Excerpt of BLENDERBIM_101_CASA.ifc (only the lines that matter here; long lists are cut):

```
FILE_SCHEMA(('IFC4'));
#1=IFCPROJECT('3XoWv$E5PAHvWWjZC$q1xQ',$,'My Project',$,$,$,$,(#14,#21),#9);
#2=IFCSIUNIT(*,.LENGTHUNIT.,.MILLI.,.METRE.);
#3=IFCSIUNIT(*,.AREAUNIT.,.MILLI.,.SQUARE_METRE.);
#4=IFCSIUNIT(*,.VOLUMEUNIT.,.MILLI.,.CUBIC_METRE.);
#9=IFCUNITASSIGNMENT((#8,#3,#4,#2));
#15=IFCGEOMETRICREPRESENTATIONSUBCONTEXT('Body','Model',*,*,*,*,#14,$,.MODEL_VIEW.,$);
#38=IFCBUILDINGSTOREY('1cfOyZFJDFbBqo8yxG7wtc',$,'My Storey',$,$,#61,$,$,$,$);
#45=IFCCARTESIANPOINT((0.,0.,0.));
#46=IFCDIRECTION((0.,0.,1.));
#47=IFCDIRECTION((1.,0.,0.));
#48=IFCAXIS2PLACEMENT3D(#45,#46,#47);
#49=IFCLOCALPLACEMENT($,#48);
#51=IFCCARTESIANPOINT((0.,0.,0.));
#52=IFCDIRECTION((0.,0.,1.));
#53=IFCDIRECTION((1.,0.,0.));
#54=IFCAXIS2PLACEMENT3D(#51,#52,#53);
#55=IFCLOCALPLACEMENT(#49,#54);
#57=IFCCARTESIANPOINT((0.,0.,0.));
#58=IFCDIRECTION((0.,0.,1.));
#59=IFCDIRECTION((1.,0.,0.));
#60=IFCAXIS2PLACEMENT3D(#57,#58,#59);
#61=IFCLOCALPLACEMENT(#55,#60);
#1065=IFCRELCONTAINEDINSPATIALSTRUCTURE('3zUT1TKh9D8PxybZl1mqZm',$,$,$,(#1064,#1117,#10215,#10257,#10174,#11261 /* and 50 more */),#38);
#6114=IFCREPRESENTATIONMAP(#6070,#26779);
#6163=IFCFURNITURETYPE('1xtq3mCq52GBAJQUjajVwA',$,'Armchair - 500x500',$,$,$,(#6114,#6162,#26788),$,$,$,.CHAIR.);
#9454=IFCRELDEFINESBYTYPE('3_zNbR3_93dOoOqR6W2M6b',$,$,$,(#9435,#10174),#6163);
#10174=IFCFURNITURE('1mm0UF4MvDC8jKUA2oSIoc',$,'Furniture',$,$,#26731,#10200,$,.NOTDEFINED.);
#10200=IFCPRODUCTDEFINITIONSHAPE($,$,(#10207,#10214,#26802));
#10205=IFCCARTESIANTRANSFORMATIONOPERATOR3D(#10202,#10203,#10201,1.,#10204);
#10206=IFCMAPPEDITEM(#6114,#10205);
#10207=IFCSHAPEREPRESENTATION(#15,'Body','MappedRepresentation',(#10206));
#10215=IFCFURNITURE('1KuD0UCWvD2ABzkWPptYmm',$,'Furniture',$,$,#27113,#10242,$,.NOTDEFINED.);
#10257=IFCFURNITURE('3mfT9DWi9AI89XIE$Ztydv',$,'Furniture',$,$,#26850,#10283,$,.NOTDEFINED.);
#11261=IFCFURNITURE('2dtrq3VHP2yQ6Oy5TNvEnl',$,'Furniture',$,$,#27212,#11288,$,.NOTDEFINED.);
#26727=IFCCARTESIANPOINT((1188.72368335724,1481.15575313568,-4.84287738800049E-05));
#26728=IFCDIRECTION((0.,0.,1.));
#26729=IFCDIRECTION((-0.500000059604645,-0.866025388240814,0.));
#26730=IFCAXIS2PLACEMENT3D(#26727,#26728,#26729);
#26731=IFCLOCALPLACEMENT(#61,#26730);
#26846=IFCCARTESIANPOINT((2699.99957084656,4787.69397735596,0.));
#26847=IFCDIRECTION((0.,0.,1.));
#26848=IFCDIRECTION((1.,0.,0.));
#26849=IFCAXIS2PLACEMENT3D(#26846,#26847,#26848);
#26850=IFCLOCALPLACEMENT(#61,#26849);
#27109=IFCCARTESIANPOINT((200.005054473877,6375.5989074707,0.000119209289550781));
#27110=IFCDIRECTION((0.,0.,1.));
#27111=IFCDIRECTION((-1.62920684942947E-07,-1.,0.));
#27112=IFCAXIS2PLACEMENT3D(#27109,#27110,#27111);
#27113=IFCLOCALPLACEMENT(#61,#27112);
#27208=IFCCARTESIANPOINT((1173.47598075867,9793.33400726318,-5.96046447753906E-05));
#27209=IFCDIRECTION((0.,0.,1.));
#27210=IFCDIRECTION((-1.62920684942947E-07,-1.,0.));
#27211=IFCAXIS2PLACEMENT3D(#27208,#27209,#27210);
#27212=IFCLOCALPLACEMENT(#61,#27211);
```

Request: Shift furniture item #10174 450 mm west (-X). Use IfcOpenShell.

```python
import ifcopenshell
import ifcopenshell.api.geometry
import ifcopenshell.util.placement

model = ifcopenshell.open("BLENDERBIM_101_CASA.ifc")

item = model.by_guid("1mm0UF4MvDC8jKUA2oSIoc")
matrix = ifcopenshell.util.placement.get_local_placement(item.ObjectPlacement)
matrix[0, 3] -= 450.0
ifcopenshell.api.geometry.edit_object_placement(model, product=item, matrix=matrix, is_si=False)

print(ifcopenshell.util.placement.get_local_placement(item.ObjectPlacement).round(3) + 0.0)

model.write("BLENDERBIM_101_CASA_v2.ifc")
```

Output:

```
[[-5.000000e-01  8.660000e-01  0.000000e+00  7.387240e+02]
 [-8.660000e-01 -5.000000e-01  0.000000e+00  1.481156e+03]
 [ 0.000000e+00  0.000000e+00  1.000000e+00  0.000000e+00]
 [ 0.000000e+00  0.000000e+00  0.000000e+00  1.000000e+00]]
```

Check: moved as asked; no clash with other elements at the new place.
